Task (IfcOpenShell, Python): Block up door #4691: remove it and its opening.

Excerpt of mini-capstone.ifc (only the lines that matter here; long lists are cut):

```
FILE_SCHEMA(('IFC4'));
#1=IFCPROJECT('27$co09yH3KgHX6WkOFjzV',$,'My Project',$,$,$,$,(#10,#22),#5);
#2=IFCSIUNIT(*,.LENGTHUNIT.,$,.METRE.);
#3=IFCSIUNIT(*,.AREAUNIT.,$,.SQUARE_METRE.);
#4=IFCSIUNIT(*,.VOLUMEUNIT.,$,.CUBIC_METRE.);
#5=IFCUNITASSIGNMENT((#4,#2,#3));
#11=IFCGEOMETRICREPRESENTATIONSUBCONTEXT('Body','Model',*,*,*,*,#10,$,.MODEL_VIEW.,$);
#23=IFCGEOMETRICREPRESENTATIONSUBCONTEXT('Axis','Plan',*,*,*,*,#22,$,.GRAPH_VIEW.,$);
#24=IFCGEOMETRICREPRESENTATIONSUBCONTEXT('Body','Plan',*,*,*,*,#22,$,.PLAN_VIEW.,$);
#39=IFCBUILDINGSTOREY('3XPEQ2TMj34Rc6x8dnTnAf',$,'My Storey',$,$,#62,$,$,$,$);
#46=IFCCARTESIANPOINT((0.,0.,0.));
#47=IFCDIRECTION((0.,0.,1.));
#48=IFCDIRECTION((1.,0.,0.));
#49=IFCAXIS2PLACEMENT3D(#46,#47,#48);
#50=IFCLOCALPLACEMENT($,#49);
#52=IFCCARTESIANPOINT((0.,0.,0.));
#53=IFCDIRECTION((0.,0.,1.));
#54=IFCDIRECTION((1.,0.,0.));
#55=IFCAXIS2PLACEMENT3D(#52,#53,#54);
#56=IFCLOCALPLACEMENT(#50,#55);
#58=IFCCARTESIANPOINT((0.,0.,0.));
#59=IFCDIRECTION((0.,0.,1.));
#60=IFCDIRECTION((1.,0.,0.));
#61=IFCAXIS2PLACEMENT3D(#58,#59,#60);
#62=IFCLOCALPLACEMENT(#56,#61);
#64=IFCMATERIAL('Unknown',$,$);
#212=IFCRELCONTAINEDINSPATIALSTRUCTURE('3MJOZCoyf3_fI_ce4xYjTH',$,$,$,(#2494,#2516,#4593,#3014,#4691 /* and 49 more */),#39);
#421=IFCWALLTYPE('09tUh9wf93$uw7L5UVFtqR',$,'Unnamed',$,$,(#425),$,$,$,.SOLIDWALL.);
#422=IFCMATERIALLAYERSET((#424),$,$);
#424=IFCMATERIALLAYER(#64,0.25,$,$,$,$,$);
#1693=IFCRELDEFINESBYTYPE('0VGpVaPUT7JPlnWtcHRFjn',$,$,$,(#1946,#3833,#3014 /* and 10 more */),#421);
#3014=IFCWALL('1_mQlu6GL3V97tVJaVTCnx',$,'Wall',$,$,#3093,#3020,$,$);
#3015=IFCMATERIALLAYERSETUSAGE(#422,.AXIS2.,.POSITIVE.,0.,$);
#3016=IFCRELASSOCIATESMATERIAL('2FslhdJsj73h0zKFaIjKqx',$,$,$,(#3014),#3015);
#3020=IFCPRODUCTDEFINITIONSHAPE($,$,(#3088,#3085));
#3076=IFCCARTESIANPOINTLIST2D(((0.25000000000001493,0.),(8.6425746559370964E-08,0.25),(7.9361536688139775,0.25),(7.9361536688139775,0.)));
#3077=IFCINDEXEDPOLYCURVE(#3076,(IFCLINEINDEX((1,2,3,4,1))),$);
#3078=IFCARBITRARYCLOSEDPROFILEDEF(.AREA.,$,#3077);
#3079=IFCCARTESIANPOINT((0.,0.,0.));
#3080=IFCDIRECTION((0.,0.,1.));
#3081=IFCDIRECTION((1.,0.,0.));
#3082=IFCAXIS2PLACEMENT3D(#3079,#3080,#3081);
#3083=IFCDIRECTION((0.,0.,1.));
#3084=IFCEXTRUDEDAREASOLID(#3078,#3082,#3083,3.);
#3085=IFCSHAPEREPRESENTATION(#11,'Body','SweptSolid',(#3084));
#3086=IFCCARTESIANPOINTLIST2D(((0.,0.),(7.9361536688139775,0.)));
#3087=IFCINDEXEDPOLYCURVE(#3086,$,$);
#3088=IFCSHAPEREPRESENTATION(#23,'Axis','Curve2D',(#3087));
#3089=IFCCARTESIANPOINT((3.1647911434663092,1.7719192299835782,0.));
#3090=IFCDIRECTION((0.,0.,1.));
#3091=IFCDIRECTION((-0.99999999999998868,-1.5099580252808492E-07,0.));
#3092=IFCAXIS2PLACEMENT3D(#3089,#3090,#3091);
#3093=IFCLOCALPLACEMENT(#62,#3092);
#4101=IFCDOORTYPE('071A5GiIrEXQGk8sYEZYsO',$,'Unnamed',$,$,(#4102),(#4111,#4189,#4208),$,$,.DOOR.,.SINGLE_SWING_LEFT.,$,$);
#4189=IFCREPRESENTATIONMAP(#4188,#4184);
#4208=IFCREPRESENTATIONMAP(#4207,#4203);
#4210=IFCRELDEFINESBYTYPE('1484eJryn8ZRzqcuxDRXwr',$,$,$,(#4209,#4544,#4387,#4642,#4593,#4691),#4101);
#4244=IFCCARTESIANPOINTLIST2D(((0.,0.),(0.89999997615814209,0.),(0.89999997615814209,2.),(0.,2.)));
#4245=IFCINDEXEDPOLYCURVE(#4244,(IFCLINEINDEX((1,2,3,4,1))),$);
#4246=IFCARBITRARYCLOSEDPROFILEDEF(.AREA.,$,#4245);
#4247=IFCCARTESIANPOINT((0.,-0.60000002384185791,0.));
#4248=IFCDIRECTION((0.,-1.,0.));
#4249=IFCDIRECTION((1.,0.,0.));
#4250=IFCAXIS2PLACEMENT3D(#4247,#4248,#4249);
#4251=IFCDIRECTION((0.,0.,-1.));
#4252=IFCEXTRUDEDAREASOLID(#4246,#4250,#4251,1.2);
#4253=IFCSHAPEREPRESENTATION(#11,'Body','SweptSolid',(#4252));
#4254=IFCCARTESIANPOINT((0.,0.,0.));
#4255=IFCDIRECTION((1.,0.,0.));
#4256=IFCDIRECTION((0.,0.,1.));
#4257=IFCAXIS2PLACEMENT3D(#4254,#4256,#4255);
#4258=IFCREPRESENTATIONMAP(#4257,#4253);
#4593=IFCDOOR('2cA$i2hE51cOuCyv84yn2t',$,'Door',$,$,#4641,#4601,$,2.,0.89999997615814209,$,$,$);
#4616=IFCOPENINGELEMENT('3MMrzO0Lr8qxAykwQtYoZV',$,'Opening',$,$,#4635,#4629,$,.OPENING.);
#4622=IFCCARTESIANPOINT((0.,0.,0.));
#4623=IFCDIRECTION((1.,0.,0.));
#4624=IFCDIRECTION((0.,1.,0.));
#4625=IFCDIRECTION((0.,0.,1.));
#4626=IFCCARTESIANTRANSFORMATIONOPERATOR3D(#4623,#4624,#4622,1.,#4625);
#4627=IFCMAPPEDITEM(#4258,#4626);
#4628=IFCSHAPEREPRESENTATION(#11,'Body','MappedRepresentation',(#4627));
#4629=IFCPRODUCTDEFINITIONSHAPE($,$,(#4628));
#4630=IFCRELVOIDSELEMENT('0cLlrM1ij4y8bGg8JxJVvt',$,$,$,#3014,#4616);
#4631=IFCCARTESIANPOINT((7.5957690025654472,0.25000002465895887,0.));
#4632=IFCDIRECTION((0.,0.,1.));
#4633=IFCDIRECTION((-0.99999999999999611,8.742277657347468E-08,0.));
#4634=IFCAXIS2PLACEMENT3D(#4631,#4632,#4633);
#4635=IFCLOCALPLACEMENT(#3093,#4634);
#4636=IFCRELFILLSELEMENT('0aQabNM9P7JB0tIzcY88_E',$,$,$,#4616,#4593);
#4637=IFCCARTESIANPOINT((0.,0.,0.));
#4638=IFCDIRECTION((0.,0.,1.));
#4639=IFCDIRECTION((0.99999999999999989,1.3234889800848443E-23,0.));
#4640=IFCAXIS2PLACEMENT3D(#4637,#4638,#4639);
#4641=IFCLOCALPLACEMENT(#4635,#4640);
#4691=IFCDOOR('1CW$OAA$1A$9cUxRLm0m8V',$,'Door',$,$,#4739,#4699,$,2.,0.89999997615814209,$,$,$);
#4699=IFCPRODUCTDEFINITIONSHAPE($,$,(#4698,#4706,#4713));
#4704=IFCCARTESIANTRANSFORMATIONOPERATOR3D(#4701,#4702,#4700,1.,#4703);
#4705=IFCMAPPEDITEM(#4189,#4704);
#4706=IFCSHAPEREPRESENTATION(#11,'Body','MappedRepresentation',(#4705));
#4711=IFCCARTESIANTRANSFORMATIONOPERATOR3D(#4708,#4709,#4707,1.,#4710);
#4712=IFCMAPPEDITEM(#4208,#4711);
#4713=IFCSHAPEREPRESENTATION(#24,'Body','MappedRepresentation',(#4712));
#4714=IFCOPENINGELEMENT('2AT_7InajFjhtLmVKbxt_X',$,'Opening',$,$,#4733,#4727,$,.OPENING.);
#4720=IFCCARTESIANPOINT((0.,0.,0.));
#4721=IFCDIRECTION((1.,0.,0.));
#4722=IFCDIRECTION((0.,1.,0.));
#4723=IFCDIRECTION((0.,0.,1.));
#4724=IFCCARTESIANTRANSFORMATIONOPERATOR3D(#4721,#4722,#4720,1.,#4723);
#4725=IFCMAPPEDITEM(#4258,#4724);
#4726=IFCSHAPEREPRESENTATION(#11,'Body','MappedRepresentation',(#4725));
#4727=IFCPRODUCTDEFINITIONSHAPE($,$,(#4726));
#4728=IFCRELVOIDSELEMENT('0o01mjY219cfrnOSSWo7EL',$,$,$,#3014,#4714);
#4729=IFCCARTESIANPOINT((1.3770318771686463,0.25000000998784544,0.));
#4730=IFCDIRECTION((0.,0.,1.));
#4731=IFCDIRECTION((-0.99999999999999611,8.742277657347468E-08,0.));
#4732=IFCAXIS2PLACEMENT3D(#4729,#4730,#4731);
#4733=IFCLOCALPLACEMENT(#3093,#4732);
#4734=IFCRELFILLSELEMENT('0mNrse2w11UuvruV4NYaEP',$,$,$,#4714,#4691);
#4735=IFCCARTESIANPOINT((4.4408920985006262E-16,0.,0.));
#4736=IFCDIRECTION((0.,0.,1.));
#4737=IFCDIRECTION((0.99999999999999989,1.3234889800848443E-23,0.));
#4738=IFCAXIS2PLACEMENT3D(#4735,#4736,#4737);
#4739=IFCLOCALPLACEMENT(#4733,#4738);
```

```python
import ifcopenshell
import ifcopenshell.api.feature
import ifcopenshell.api.root
import ifcopenshell.geom
import ifcopenshell.util.shape

model = ifcopenshell.open("mini-capstone.ifc")
settings = ifcopenshell.geom.settings()


def volume(element):
    """Net volume in cubic metres, openings subtracted."""
    shape = ifcopenshell.geom.create_shape(settings, element)
    return ifcopenshell.util.shape.get_volume(shape.geometry)


door = model.by_guid("1CW$OAA$1A$9cUxRLm0m8V")
opening = door.FillsVoids[0].RelatingOpeningElement
wall = opening.VoidsElements[0].RelatingBuildingElement
before = volume(wall)

ifcopenshell.api.root.remove_product(model, product=door)
ifcopenshell.api.feature.remove_feature(model, feature=opening)

after = volume(wall)

print(f"wall volume {before:.3f} -> {after:.3f} m3")

model.write("mini-capstone_edited.ifc")
```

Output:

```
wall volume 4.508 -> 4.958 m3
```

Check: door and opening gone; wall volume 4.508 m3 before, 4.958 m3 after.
